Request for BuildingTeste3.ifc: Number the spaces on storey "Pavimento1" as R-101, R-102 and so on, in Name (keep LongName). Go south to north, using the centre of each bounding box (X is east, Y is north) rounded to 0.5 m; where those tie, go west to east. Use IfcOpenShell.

First a look at what the model holds.

```python
import ifcopenshell
import ifcopenshell.util.element
import ifcopenshell.util.placement

model = ifcopenshell.open("BuildingTeste3.ifc")
print(model.schema)
storey = next(s for s in model.by_type("IfcBuildingStorey") if s.Name == "Pavimento1")
spaces = [e for e in ifcopenshell.util.element.get_decomposition(storey) if e.is_a("IfcSpace")]
for e in sorted(spaces, key=lambda e: e.id()):
    origin = ifcopenshell.util.placement.get_local_placement(e.ObjectPlacement)[:3, 3]
    print(e.id(), e.Name, e.LongName, origin.round(2) + 0.0, sep=" | ")
```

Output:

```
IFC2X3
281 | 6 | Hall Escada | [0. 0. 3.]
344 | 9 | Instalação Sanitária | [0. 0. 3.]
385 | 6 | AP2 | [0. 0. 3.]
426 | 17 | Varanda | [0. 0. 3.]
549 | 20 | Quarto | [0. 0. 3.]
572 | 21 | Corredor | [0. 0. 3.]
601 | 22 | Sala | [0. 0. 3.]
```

```python
import ifcopenshell
import ifcopenshell.geom
import ifcopenshell.util.element
import ifcopenshell.util.shape

model = ifcopenshell.open("BuildingTeste3.ifc")
settings = ifcopenshell.geom.settings()
settings.set("use-world-coords", True)


def centre(element):
    shape = ifcopenshell.geom.create_shape(settings, element)
    return ifcopenshell.util.shape.get_bbox_centroid(shape.geometry)


storey = next(s for s in model.by_type("IfcBuildingStorey") if s.Name == "Pavimento1")
spaces = [e for e in ifcopenshell.util.element.get_decomposition(storey) if e.is_a("IfcSpace")]

# Insertion points can sit at a corner or the storey origin, so sort by the geometry (in metres).
centres = {e: centre(e) for e in spaces}
spaces.sort(key=lambda e: (round(centres[e][1] / 0.5), centres[e][0]))

for i, e in enumerate(spaces, start=1):
    number = f"R-1{i:02d}"
    e.Name = number
    print(e.id(), number)

model.write("BuildingTeste3-out.ifc")
```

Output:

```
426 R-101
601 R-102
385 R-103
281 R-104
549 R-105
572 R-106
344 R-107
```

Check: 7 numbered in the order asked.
